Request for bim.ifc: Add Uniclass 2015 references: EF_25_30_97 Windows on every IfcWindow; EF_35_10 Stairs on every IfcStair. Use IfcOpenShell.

First a look at what the model holds.

```python
import ifcopenshell

model = ifcopenshell.open("bim.ifc")
print(model.schema)
print("classifications:", [c.Name for c in model.by_type("IfcClassification")])
for ifc_class in ("IfcDoor", "IfcRoof", "IfcStair", "IfcWall", "IfcWindow"):
    print(ifc_class, len(model.by_type(ifc_class)))
```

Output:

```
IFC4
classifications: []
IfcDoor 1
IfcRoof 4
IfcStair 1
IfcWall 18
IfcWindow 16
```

```python
import ifcopenshell
import ifcopenshell.api.classification

model = ifcopenshell.open("bim.ifc")

system = ifcopenshell.api.classification.add_classification(model, classification="Uniclass 2015")

codes = {
    "IfcWindow": ("EF_25_30_97", "Windows"),
    "IfcStair": ("EF_35_10", "Stairs"),
}
for ifc_class, (code, name) in codes.items():
    products = model.by_type(ifc_class)
    ifcopenshell.api.classification.add_reference(
        model, products=products, classification=system, identification=code, name=name
    )
    print(code, len(products))

model.write("bim_edited.ifc")
```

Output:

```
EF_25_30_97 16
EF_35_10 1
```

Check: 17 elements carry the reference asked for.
